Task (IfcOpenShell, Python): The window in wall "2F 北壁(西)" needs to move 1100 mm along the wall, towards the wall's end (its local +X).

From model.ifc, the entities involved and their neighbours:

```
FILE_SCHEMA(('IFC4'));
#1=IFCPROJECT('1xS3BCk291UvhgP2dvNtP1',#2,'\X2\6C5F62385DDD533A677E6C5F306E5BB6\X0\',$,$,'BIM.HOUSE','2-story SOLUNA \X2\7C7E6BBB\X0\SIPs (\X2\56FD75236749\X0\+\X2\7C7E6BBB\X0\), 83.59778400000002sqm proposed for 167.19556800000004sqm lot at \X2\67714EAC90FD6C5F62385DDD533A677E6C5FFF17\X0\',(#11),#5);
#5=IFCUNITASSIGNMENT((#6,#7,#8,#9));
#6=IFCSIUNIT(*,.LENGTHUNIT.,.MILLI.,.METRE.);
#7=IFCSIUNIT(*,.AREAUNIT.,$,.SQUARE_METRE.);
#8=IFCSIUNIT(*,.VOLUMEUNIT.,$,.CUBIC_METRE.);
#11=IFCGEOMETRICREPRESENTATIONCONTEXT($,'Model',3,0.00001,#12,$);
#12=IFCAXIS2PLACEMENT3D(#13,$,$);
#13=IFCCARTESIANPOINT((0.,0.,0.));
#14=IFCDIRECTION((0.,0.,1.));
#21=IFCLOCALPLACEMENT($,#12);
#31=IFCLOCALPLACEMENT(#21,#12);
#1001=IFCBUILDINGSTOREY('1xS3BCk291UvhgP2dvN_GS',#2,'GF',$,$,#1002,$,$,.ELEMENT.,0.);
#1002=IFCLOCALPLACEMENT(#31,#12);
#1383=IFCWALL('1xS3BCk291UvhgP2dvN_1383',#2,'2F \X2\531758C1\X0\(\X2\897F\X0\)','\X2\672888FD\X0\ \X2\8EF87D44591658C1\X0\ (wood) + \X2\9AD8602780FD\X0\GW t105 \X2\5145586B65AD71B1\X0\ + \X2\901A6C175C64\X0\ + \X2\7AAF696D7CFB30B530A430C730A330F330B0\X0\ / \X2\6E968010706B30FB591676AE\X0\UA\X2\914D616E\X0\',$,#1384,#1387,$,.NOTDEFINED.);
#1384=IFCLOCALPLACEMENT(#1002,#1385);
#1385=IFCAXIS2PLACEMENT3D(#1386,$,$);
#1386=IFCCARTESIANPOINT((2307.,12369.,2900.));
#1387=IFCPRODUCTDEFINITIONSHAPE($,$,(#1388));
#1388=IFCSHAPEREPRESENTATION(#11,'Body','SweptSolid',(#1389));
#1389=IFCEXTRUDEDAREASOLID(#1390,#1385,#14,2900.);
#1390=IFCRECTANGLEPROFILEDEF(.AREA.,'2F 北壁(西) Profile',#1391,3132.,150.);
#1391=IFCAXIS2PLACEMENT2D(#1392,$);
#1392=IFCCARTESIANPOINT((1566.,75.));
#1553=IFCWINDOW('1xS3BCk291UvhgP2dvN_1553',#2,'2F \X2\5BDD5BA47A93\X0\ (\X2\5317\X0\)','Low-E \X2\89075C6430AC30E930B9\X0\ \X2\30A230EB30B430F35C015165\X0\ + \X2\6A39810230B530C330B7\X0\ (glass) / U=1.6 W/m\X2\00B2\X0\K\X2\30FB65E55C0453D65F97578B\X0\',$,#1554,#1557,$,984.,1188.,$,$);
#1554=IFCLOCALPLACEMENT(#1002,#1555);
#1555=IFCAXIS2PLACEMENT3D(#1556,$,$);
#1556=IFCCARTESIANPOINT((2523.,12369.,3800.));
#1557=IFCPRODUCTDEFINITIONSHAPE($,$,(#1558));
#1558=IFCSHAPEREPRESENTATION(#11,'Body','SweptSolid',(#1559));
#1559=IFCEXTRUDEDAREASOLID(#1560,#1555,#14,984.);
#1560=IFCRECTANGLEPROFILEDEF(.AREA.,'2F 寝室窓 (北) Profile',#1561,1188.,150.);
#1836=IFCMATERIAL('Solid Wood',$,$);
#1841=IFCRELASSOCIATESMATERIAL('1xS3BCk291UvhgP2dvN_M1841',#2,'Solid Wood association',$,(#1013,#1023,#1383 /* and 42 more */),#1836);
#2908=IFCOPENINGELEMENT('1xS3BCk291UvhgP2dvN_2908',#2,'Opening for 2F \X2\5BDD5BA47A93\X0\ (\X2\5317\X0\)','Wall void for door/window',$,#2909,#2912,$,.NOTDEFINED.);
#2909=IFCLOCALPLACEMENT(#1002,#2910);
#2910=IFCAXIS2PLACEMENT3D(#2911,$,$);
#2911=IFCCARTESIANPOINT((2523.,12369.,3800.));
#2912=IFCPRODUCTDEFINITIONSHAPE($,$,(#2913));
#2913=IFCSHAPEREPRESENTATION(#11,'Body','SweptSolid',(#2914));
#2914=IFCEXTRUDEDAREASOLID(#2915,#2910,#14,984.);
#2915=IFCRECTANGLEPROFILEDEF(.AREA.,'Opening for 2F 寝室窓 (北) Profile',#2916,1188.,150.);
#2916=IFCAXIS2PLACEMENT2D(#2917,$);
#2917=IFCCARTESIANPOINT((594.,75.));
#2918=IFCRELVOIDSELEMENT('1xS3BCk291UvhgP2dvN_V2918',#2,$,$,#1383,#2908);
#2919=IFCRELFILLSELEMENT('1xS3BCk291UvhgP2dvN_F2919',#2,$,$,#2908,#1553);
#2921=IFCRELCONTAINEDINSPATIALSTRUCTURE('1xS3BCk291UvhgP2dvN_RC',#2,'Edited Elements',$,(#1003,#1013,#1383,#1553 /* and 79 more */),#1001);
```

```python
import ifcopenshell
import ifcopenshell.api.geometry
import ifcopenshell.util.placement

model = ifcopenshell.open("model.ifc")

window = model.by_guid("1xS3BCk291UvhgP2dvN_1553")
opening = window.FillsVoids[0].RelatingOpeningElement
wall = opening.VoidsElements[0].RelatingBuildingElement

wall_matrix = ifcopenshell.util.placement.get_local_placement(wall.ObjectPlacement)
shift = wall_matrix[:3, 0] * 1100.0
before = ifcopenshell.util.placement.get_local_placement(window.ObjectPlacement)[:3, 3].copy()

# The window is not placed relative to its opening, so move both.
for product in (opening, window):
    matrix = ifcopenshell.util.placement.get_local_placement(product.ObjectPlacement)
    matrix[:3, 3] += shift
    ifcopenshell.api.geometry.edit_object_placement(model, product=product, matrix=matrix, is_si=False)

after = ifcopenshell.util.placement.get_local_placement(window.ObjectPlacement)[:3, 3]
print("window moved by", (after - before).round(3) + 0.0)

model.write("model_edited.ifc")
```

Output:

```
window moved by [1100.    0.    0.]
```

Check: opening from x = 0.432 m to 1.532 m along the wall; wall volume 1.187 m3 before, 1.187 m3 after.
